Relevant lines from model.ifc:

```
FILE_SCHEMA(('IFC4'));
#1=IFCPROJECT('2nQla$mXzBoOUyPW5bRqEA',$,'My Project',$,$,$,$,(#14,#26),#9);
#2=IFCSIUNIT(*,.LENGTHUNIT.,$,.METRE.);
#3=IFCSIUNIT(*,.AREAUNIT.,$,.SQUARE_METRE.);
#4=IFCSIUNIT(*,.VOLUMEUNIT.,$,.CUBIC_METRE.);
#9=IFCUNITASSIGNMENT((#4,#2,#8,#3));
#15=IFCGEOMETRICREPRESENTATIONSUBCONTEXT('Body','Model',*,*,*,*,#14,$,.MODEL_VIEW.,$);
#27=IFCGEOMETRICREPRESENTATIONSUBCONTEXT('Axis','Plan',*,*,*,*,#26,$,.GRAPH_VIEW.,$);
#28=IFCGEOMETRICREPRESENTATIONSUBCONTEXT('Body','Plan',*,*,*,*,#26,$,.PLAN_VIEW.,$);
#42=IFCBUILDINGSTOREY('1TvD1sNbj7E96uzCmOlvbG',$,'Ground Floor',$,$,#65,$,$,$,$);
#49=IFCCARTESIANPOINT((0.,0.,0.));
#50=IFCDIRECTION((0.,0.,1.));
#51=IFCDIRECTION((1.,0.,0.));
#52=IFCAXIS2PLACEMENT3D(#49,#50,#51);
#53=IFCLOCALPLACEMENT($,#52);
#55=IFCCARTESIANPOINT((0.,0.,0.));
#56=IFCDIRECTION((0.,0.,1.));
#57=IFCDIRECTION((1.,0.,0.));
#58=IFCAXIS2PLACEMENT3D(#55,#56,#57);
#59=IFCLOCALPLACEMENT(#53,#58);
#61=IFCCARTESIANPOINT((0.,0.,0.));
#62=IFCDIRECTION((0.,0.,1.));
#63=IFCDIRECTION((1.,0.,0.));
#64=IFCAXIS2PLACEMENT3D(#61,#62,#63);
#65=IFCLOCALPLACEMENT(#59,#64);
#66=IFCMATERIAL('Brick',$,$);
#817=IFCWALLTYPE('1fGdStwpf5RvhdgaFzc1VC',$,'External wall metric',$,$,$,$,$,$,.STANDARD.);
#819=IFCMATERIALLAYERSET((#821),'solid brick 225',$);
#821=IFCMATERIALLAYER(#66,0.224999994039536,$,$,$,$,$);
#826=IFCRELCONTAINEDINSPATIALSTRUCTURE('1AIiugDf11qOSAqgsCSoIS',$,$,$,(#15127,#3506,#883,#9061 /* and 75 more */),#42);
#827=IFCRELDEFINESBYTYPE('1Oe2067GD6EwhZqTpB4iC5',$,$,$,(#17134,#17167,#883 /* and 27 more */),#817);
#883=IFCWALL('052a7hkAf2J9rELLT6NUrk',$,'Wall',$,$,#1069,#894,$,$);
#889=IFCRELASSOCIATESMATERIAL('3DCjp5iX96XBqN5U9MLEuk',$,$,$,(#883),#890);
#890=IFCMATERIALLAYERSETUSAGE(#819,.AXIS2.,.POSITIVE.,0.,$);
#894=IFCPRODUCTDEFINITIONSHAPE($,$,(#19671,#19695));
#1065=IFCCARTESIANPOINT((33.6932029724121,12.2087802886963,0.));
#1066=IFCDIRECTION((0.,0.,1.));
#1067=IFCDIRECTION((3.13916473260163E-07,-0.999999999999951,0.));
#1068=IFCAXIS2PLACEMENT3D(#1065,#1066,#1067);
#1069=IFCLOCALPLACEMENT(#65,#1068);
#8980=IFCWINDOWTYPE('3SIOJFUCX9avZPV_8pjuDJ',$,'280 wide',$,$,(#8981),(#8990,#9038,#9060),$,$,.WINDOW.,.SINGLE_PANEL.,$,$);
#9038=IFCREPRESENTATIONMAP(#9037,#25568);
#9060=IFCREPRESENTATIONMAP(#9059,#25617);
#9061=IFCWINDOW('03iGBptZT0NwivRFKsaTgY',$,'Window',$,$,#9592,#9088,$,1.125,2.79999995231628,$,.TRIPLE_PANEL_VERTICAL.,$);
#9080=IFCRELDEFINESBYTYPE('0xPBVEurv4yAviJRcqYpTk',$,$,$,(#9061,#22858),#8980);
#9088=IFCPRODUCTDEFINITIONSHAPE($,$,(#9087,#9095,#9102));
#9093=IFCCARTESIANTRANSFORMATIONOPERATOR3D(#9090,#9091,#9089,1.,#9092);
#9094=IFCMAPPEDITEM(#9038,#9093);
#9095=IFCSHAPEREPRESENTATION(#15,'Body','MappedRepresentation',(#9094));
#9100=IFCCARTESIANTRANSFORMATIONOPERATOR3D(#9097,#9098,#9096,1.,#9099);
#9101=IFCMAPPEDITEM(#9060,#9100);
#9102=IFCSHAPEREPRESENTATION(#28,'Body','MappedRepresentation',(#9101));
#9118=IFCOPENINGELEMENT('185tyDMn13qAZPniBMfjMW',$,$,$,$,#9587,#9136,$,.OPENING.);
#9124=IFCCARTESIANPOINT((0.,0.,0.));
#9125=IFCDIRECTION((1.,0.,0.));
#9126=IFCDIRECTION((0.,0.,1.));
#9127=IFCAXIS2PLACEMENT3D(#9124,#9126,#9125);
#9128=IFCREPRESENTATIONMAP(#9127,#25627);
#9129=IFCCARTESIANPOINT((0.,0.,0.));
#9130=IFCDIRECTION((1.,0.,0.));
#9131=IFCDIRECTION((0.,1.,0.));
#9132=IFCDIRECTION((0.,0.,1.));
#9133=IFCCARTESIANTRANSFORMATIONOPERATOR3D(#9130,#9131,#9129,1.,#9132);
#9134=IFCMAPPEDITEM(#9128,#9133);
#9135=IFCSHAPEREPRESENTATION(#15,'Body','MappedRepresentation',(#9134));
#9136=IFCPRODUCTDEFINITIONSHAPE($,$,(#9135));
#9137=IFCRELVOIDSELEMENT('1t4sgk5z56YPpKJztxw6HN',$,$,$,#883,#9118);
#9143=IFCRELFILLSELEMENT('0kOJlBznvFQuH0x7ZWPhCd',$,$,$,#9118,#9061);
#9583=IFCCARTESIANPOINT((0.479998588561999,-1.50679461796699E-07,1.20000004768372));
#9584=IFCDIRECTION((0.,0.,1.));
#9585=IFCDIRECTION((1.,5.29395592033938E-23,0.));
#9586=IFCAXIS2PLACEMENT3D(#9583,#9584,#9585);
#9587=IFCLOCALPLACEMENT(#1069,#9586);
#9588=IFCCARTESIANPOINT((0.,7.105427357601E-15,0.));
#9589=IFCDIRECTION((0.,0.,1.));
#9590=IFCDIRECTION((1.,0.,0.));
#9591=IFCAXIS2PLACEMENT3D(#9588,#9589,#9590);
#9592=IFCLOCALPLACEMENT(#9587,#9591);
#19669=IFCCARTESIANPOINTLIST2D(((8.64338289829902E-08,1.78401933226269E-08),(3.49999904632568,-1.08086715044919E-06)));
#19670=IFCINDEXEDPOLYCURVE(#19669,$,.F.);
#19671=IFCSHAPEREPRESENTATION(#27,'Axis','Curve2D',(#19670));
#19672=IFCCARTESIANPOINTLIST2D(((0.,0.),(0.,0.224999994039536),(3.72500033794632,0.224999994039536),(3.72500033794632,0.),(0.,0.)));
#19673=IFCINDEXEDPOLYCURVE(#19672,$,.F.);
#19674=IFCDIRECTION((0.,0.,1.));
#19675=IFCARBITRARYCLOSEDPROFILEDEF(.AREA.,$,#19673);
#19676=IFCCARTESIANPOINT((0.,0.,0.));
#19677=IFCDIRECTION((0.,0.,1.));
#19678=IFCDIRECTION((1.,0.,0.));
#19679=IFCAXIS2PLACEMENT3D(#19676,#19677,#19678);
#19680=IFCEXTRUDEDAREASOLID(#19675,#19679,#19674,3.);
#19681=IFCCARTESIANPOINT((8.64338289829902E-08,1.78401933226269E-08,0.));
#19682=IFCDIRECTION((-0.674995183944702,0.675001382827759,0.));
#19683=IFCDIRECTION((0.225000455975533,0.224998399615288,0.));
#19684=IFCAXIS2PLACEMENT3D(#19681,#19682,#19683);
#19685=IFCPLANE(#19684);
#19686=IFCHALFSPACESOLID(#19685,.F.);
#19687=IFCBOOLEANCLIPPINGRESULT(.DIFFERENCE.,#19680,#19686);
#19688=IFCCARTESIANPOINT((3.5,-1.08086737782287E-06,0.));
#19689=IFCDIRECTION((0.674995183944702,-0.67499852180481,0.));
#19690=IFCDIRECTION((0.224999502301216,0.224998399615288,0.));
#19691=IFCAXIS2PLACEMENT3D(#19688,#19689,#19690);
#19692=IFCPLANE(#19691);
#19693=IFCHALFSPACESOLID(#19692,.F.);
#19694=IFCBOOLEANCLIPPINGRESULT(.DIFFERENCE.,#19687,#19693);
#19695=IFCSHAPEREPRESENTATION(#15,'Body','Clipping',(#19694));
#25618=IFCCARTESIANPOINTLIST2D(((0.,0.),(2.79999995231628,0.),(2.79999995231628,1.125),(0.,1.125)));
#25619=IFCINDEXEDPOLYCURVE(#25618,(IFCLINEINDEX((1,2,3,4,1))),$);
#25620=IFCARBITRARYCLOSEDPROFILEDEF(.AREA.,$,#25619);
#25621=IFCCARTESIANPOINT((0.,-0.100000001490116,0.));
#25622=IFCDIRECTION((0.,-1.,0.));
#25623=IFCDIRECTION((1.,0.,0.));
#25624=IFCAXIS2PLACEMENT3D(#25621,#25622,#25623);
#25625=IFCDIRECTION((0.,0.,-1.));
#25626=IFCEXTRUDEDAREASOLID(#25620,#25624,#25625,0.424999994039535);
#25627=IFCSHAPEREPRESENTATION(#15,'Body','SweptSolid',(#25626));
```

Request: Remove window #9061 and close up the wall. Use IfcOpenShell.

```python
import ifcopenshell
import ifcopenshell.api.feature
import ifcopenshell.api.root
import ifcopenshell.geom
import ifcopenshell.util.shape

model = ifcopenshell.open("model.ifc")
settings = ifcopenshell.geom.settings()


def volume(element):
    """Net volume in cubic metres, openings subtracted."""
    shape = ifcopenshell.geom.create_shape(settings, element)
    return ifcopenshell.util.shape.get_volume(shape.geometry)


window = model.by_guid("03iGBptZT0NwivRFKsaTgY")
opening = window.FillsVoids[0].RelatingOpeningElement
wall = opening.VoidsElements[0].RelatingBuildingElement
before = volume(wall)

ifcopenshell.api.root.remove_product(model, product=window)
ifcopenshell.api.feature.remove_feature(model, feature=opening)

after = volume(wall)

print(f"wall volume {before:.3f} -> {after:.3f} m3")

model.write("model_rev.ifc")
```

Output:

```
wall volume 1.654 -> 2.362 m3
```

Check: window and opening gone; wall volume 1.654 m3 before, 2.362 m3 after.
